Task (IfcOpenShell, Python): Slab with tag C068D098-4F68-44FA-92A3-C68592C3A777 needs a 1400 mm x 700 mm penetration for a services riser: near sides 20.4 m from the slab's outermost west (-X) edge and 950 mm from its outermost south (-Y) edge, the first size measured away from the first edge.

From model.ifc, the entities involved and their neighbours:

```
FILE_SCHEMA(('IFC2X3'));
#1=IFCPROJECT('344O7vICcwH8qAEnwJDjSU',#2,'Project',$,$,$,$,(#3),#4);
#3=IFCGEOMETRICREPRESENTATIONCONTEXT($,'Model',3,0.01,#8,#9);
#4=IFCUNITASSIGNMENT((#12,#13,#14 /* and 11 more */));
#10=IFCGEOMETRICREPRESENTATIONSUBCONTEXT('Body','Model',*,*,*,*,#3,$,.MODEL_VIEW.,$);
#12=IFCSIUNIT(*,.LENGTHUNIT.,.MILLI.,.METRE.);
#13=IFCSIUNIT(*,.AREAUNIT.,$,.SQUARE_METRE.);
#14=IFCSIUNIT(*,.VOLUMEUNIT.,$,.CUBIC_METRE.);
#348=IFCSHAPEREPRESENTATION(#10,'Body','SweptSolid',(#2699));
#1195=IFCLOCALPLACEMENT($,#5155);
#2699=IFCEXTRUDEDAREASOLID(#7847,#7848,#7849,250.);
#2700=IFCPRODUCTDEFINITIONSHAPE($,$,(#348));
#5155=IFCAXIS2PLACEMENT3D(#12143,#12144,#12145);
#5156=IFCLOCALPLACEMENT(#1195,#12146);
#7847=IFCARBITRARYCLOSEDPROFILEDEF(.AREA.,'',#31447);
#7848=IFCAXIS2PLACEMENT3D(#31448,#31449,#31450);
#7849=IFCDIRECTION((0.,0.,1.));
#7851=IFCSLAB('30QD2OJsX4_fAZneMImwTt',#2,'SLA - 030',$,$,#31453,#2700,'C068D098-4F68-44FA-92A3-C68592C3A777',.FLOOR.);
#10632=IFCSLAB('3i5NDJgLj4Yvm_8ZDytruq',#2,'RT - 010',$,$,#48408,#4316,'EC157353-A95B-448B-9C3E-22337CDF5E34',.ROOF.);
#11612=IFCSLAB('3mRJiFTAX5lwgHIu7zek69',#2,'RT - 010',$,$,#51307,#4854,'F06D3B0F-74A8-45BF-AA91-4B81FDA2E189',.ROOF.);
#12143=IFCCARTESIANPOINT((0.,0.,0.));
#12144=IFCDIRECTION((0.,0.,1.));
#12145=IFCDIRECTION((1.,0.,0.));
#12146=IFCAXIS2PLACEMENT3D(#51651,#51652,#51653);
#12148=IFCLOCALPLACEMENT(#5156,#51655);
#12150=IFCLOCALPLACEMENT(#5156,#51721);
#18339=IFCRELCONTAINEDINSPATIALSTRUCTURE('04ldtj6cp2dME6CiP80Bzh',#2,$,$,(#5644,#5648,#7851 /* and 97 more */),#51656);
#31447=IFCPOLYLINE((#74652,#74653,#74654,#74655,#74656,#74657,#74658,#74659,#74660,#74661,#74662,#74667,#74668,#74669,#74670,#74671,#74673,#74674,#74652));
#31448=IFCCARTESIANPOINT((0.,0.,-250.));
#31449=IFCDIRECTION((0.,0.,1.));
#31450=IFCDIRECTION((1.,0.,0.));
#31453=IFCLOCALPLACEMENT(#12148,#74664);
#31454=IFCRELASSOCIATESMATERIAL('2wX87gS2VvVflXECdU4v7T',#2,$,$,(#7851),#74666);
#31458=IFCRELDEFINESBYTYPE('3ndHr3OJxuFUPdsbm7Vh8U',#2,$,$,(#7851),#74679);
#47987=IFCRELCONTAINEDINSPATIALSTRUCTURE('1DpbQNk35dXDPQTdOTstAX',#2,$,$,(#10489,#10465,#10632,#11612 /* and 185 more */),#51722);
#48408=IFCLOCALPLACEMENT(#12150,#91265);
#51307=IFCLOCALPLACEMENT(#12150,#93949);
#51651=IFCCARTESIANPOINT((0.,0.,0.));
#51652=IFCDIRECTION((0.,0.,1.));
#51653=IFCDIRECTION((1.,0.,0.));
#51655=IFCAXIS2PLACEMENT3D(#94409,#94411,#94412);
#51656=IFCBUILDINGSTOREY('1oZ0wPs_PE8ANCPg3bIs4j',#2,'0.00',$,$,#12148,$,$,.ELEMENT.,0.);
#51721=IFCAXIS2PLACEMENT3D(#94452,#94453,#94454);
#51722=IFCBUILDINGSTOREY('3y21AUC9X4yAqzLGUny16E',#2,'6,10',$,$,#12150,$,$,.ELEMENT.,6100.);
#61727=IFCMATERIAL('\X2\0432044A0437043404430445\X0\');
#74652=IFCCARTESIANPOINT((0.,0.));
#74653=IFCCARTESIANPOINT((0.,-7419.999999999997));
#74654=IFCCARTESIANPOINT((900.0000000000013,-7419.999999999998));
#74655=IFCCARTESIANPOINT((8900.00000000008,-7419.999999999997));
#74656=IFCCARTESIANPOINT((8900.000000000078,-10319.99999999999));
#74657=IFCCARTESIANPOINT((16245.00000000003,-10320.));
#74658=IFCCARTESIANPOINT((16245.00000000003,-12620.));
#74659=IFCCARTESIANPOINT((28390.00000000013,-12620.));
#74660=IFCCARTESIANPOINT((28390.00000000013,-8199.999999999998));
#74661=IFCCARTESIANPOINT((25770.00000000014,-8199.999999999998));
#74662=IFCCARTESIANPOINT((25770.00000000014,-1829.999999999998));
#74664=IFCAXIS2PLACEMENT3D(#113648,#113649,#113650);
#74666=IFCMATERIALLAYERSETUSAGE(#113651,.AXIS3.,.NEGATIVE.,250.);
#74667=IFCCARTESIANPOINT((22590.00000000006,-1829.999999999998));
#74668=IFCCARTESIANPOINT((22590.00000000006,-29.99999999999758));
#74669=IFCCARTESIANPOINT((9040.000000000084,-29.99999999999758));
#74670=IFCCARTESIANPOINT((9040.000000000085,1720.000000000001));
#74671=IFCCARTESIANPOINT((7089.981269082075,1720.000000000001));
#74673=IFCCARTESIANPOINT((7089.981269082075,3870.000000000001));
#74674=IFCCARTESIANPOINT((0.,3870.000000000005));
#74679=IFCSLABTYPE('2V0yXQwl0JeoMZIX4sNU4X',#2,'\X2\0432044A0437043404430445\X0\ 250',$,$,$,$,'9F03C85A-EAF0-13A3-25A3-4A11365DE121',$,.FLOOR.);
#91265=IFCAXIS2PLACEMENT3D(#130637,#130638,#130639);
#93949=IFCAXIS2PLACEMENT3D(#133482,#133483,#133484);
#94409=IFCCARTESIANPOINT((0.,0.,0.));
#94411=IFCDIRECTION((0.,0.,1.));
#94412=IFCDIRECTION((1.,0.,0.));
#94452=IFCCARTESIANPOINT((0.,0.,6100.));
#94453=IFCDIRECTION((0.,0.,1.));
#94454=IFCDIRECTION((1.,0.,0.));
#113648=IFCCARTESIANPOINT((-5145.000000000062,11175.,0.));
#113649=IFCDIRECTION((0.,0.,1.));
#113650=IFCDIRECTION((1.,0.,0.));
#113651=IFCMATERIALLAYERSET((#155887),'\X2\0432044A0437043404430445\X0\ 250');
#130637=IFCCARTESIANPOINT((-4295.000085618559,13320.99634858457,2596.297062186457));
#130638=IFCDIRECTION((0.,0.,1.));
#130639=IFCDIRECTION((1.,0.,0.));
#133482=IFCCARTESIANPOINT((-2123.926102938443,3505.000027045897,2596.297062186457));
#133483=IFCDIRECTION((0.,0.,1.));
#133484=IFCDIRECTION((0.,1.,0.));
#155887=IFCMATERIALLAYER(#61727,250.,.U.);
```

```python
import numpy as np
import ifcopenshell
import ifcopenshell.api.feature
import ifcopenshell.api.geometry
import ifcopenshell.api.root
import ifcopenshell.geom
import ifcopenshell.util.placement
import ifcopenshell.util.representation
import ifcopenshell.util.shape
import ifcopenshell.util.unit

model = ifcopenshell.open("model.ifc")
unit_scale = ifcopenshell.util.unit.calculate_unit_scale(model)
settings = ifcopenshell.geom.settings()


def volume(element):
    """Net volume in cubic metres, openings subtracted."""
    shape = ifcopenshell.geom.create_shape(settings, element)
    return ifcopenshell.util.shape.get_volume(shape.geometry)


slab = model.by_guid("30QD2OJsX4_fAZneMImwTt")
before = volume(slab)

# Extent in the slab's own axes, in metres. The edges named are its -X and -Y sides.
slab_shape = ifcopenshell.geom.create_shape(settings, slab)
vertices = ifcopenshell.util.shape.get_vertices(slab_shape.geometry)
x_min, y_min, bottom = vertices.min(axis=0)
top = vertices[:, 2].max()

opening = ifcopenshell.api.root.create_entity(model, ifc_class="IfcOpeningElement", name="Services riser opening")
context = ifcopenshell.util.representation.get_context(model, "Model", "Body", "MODEL_VIEW")
width, depth = 1.4, 0.7
outline = [(0.0, 0.0), (width, 0.0), (width, depth), (0.0, depth), (0.0, 0.0)]
# Overshoot both faces by 50 mm so the cut is clean.
shape = ifcopenshell.api.geometry.add_slab_representation(
    model, context=context, depth=top - bottom + 0.1, polyline=outline
)
ifcopenshell.api.geometry.assign_representation(model, product=opening, representation=shape)

matrix = ifcopenshell.util.placement.get_local_placement(slab.ObjectPlacement)
matrix[:, 3] = matrix @ np.append(np.array([x_min + 20.4, y_min + 0.95, bottom - 0.05]) / unit_scale, 1.0)
ifcopenshell.api.geometry.edit_object_placement(model, product=opening, matrix=matrix, is_si=False)
ifcopenshell.api.feature.add_feature(model, feature=opening, element=slab)

after = volume(slab)

print(f"slab volume {before:.3f} -> {after:.3f} m3")

model.write("model_updated.ifc")
```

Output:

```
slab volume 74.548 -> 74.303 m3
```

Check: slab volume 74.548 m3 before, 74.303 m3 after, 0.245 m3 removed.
